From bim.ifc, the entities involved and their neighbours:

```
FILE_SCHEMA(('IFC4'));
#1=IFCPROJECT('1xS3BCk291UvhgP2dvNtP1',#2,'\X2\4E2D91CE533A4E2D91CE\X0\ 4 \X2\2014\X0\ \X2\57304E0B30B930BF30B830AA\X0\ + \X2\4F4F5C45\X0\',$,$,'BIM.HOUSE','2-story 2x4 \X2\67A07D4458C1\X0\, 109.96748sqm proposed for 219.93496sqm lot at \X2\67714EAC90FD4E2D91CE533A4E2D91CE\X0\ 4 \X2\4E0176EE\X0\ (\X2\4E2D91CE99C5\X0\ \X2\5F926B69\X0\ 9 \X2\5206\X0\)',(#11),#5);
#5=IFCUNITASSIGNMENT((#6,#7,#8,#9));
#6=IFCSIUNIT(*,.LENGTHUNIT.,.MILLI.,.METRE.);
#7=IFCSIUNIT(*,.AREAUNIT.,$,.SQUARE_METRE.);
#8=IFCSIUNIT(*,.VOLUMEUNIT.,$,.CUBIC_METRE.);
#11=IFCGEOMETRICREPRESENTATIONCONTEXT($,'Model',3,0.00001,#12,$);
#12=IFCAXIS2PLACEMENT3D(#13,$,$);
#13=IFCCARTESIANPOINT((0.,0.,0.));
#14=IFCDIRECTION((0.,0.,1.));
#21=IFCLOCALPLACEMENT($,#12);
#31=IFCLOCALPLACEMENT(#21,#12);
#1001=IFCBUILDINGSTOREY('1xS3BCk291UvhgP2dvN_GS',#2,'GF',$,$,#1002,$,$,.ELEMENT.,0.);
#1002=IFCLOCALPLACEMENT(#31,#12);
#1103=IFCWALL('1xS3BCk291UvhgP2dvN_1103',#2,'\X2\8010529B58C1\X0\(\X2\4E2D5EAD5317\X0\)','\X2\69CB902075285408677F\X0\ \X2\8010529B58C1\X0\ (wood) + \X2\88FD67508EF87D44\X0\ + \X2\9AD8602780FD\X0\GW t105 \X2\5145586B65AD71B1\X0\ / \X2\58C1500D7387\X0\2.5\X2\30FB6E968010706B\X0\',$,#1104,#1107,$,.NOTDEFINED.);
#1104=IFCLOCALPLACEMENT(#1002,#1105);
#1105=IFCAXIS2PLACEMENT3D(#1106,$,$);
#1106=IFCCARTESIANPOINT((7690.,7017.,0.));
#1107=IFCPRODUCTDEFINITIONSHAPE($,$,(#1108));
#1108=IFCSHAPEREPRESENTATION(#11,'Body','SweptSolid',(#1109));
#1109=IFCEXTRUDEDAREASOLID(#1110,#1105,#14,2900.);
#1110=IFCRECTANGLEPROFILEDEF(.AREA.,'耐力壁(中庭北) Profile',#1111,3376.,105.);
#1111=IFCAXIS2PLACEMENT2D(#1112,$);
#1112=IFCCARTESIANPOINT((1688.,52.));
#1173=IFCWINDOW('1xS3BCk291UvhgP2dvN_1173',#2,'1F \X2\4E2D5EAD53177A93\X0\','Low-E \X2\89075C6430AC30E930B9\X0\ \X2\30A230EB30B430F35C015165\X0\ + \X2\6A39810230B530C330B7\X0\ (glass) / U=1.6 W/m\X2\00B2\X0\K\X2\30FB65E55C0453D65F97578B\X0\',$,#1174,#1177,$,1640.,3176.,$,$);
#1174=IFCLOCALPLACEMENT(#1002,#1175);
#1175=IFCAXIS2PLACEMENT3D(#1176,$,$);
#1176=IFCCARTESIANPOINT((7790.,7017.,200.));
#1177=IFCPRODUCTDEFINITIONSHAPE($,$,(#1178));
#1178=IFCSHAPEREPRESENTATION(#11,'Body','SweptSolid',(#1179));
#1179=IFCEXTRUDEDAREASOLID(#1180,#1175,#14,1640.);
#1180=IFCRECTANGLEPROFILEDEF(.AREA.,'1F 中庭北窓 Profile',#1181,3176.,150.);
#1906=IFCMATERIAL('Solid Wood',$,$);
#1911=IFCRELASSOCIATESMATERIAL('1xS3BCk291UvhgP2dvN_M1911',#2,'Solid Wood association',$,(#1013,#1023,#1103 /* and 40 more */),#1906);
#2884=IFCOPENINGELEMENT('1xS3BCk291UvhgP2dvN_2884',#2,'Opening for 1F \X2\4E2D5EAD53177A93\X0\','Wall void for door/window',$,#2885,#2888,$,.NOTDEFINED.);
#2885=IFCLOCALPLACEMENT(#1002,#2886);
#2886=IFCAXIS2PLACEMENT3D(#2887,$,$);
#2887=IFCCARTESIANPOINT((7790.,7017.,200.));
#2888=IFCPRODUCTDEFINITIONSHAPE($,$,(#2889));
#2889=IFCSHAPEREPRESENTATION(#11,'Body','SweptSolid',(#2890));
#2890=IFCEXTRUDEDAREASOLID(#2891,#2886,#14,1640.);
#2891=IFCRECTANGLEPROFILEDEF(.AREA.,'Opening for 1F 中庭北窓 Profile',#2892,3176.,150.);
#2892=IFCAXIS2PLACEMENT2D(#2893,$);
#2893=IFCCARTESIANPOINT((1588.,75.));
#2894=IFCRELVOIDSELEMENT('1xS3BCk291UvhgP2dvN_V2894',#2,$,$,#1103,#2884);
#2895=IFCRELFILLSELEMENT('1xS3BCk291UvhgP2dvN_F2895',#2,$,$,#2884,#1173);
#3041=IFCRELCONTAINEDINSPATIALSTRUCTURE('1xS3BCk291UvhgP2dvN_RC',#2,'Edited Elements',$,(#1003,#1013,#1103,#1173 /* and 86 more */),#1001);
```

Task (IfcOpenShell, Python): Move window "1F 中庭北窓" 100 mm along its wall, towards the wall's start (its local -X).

```python
import ifcopenshell
import ifcopenshell.api.geometry
import ifcopenshell.util.placement

model = ifcopenshell.open("bim.ifc")

window = model.by_guid("1xS3BCk291UvhgP2dvN_1173")
opening = window.FillsVoids[0].RelatingOpeningElement
wall = opening.VoidsElements[0].RelatingBuildingElement

wall_matrix = ifcopenshell.util.placement.get_local_placement(wall.ObjectPlacement)
shift = wall_matrix[:3, 0] * -100.0
before = ifcopenshell.util.placement.get_local_placement(window.ObjectPlacement)[:3, 3].copy()

# The window is not placed relative to its opening, so move both.
for product in (opening, window):
    matrix = ifcopenshell.util.placement.get_local_placement(product.ObjectPlacement)
    matrix[:3, 3] += shift
    ifcopenshell.api.geometry.edit_object_placement(model, product=product, matrix=matrix, is_si=False)

after = ifcopenshell.util.placement.get_local_placement(window.ObjectPlacement)[:3, 3]
print("window moved by", (after - before).round(3) + 0.0)

model.write("bim_rev.ifc")
```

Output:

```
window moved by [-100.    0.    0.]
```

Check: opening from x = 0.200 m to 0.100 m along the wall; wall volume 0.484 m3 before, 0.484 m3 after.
